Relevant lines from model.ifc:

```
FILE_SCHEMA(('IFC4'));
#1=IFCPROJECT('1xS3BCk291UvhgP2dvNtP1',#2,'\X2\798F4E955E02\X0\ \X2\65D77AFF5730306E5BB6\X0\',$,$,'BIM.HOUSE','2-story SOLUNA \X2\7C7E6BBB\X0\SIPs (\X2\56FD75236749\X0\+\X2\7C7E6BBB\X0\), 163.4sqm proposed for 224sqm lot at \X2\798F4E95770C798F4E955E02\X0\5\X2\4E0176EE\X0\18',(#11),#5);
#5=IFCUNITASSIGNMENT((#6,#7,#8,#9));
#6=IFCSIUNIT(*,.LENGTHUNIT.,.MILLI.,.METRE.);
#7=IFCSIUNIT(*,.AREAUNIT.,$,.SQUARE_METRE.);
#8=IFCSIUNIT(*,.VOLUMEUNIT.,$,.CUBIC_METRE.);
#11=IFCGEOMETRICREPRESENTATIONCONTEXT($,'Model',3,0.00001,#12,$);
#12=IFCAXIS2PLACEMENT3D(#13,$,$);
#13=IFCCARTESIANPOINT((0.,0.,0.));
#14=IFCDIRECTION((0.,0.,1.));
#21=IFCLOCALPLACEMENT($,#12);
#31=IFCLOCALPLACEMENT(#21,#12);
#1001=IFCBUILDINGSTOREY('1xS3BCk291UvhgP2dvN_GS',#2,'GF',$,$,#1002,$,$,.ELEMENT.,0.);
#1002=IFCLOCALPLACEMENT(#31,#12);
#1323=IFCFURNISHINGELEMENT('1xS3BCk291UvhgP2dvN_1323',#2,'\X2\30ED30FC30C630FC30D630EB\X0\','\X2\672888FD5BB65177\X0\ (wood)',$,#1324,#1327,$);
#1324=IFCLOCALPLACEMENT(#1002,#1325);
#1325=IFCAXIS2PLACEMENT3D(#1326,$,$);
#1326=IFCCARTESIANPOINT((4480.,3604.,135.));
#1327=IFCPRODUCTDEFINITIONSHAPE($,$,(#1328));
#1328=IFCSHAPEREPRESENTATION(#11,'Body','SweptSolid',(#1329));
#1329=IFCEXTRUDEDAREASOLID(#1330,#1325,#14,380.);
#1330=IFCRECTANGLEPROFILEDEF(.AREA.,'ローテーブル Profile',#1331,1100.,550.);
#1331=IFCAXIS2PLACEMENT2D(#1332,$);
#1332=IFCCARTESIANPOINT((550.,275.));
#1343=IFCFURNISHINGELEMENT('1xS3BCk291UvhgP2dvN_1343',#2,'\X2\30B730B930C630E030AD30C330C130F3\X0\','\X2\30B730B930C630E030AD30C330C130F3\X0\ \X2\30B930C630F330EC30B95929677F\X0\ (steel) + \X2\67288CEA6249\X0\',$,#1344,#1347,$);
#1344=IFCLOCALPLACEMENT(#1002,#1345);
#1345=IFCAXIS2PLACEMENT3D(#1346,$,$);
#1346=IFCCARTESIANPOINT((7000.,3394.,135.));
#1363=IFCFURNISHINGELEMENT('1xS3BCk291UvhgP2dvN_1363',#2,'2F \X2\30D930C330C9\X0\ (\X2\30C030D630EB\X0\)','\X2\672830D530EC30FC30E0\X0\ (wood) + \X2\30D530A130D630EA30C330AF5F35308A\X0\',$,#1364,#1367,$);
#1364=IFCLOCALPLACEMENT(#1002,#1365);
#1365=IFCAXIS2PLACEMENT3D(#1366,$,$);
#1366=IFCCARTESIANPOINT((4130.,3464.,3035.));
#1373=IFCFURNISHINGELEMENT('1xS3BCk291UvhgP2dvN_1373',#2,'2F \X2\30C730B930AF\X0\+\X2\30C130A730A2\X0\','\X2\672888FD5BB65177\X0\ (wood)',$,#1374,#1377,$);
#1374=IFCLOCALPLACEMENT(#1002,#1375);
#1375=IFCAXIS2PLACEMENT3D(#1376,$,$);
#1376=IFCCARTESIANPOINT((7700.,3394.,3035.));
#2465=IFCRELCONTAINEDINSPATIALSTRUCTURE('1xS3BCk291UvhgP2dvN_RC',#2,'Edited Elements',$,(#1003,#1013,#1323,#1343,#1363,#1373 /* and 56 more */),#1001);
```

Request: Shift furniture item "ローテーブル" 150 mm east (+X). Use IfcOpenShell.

```python
import ifcopenshell
import ifcopenshell.api.geometry
import ifcopenshell.util.placement
import ifcopenshell.util.unit

model = ifcopenshell.open("model.ifc")
unit_scale = ifcopenshell.util.unit.calculate_unit_scale(model)

item = model.by_guid("1xS3BCk291UvhgP2dvN_1323")
matrix = ifcopenshell.util.placement.get_local_placement(item.ObjectPlacement)
matrix[0, 3] += 0.15 / unit_scale
ifcopenshell.api.geometry.edit_object_placement(model, product=item, matrix=matrix, is_si=False)

print(ifcopenshell.util.placement.get_local_placement(item.ObjectPlacement).round(3) + 0.0)

model.write("model_updated.ifc")
```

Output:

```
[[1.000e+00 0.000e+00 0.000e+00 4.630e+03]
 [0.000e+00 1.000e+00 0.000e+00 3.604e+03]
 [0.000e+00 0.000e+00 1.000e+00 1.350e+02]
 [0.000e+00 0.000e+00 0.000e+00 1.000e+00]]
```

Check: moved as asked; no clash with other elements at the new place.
